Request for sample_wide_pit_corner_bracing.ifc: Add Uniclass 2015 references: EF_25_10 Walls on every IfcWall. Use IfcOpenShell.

First a look at what the model holds.

```python
import ifcopenshell

model = ifcopenshell.open("sample_wide_pit_corner_bracing.ifc")
print(model.schema)
print("classifications:", [c.Name for c in model.by_type("IfcClassification")])
for ifc_class in ("IfcDoor", "IfcRoof", "IfcStair", "IfcWall", "IfcWindow"):
    print(ifc_class, len(model.by_type(ifc_class)))
```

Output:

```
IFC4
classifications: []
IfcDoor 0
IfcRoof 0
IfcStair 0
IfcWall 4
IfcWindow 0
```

```python
import ifcopenshell
import ifcopenshell.api.classification

model = ifcopenshell.open("sample_wide_pit_corner_bracing.ifc")

system = ifcopenshell.api.classification.add_classification(model, classification="Uniclass 2015")

codes = {
    "IfcWall": ("EF_25_10", "Walls"),
}
for ifc_class, (code, name) in codes.items():
    products = model.by_type(ifc_class)
    ifcopenshell.api.classification.add_reference(
        model, products=products, classification=system, identification=code, name=name
    )
    print(code, len(products))

model.write("sample_wide_pit_corner_bracing_v2.ifc")
```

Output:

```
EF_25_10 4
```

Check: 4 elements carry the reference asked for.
